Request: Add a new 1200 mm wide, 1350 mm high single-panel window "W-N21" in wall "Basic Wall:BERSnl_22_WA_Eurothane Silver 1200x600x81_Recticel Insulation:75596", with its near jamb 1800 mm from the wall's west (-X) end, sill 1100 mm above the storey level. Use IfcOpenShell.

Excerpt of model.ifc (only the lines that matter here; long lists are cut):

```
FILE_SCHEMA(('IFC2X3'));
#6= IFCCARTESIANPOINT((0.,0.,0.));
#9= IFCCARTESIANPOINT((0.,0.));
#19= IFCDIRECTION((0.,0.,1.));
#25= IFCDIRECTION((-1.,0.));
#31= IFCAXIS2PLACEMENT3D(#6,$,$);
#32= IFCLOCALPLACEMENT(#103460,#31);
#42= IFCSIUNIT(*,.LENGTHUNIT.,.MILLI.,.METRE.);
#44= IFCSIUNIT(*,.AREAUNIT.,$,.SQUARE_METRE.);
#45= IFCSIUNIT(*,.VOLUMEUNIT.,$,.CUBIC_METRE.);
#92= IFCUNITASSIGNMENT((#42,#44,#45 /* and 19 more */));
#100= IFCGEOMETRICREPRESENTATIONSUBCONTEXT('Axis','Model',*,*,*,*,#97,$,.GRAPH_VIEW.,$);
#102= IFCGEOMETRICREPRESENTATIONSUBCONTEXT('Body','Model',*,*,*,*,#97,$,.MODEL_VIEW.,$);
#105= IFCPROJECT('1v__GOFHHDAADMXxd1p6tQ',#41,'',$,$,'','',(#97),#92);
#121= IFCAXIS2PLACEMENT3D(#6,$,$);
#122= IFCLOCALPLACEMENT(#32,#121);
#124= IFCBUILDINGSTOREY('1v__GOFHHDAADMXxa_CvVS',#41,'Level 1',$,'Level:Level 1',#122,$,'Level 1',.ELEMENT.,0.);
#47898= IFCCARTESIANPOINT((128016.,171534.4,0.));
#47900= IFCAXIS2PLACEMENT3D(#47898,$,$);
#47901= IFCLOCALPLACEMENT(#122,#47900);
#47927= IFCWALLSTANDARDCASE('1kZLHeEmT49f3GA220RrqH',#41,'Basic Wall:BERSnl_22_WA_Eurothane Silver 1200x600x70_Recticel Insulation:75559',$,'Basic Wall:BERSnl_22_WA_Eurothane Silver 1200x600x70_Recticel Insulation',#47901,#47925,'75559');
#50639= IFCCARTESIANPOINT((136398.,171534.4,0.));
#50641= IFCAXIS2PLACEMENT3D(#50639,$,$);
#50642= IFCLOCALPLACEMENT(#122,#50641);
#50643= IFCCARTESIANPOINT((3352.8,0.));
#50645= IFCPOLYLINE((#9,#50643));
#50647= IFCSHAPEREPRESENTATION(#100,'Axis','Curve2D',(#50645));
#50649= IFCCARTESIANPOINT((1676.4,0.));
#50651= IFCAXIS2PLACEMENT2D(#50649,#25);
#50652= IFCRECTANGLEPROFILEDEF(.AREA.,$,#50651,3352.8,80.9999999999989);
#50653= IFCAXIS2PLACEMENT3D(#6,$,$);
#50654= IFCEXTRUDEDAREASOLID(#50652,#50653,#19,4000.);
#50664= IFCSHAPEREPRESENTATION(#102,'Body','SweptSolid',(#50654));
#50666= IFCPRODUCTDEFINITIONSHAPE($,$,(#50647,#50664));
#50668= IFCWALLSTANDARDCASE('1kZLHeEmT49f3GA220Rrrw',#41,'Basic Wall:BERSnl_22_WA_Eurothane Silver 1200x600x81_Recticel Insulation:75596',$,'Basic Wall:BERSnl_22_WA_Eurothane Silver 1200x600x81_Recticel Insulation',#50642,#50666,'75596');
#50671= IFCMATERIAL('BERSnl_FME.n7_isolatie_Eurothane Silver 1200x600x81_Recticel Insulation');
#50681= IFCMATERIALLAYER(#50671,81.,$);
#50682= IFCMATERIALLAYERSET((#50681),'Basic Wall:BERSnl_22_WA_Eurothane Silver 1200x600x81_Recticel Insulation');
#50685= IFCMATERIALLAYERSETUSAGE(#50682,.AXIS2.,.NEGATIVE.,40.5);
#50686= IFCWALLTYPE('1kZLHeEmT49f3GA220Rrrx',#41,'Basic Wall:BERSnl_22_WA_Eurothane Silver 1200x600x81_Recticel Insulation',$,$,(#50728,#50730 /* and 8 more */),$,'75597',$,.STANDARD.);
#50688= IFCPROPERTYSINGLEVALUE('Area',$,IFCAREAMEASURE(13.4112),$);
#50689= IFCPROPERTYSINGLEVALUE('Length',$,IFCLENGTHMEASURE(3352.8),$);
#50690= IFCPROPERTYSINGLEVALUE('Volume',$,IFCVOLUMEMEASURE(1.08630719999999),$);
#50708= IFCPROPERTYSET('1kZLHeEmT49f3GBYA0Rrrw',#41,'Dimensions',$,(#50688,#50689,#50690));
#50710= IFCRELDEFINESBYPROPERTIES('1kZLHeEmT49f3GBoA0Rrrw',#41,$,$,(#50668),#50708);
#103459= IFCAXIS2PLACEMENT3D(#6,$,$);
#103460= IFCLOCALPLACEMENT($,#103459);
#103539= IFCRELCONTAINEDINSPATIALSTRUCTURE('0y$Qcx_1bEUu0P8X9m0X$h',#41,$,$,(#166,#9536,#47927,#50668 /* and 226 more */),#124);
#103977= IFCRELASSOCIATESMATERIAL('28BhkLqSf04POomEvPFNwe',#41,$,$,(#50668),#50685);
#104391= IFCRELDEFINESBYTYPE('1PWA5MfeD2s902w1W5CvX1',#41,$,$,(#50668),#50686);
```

```python
import numpy as np
import ifcopenshell
import ifcopenshell.api.feature
import ifcopenshell.api.geometry
import ifcopenshell.api.pset
import ifcopenshell.api.root
import ifcopenshell.api.spatial
import ifcopenshell.api.type
import ifcopenshell.geom
import ifcopenshell.util.element
import ifcopenshell.util.placement
import ifcopenshell.util.representation
import ifcopenshell.util.shape
import ifcopenshell.util.unit

model = ifcopenshell.open("model.ifc")
unit_scale = ifcopenshell.util.unit.calculate_unit_scale(model)
area_scale = ifcopenshell.util.unit.calculate_unit_scale(model, "AREAUNIT")
volume_scale = ifcopenshell.util.unit.calculate_unit_scale(model, "VOLUMEUNIT")
settings = ifcopenshell.geom.settings()


def volume(element):
    """Net volume in cubic metres, openings subtracted."""
    shape = ifcopenshell.geom.create_shape(settings, element)
    return ifcopenshell.util.shape.get_volume(shape.geometry)


wall = model.by_guid("1kZLHeEmT49f3GA220Rrrw")
storey = ifcopenshell.util.element.get_container(wall, ifc_class="IfcBuildingStorey")
context = ifcopenshell.util.representation.get_context(model, "Model", "Body", "MODEL_VIEW")
before = volume(wall)

width, height, from_end, sill = 1.2, 1.35, 1.8, 1.1  # metres

# The wall runs along its own X axis, and the end named is its -X end.
wall_shape = ifcopenshell.geom.create_shape(settings, wall)
x, y, z = ifcopenshell.util.shape.get_vertices(wall_shape.geometry).T
start = x.min() + from_end
face, thickness = float(y.min()), float(y.max() - y.min())
wall_matrix = ifcopenshell.util.placement.get_local_placement(wall.ObjectPlacement)
level = ifcopenshell.util.placement.get_local_placement(storey.ObjectPlacement)[2, 3]


def in_wall(x, y):
    """Placement at x, y metres in the wall's axes, at sill height."""
    matrix = wall_matrix.copy()
    matrix[:, 3] = wall_matrix @ np.array([x / unit_scale, y / unit_scale, 0.0, 1.0])
    matrix[2, 3] = level + sill / unit_scale
    return matrix


# Opening: a box that overshoots both wall faces by 50 mm.
opening = ifcopenshell.api.root.create_entity(model, ifc_class="IfcOpeningElement")
box = ifcopenshell.api.geometry.add_wall_representation(
    model, context=context, length=width, height=height, thickness=thickness + 0.1
)
ifcopenshell.api.geometry.assign_representation(model, product=opening, representation=box)
ifcopenshell.api.geometry.edit_object_placement(model, product=opening, matrix=in_wall(start, face - 0.05), is_si=False)
ifcopenshell.api.feature.add_feature(model, feature=opening, element=wall)

window = ifcopenshell.api.root.create_entity(model, ifc_class="IfcWindow", name="W-N21")
window.OverallWidth, window.OverallHeight = width / unit_scale, height / unit_scale
body = ifcopenshell.api.geometry.add_window_representation(
    model,
    context=context,
    overall_width=window.OverallWidth,
    overall_height=window.OverallHeight,
    partition_type="SINGLE_PANEL",
)
ifcopenshell.api.geometry.assign_representation(model, product=window, representation=body)
ifcopenshell.api.spatial.assign_container(model, products=[window], relating_structure=storey)
fills = ifcopenshell.api.feature.add_filling(model, opening=opening, element=window)
fills.OwnerHistory = window.OwnerHistory  # required in IFC2X3

# IFC2X3 keeps the operation on the window style.
style = ifcopenshell.api.root.create_entity(model, ifc_class="IfcWindowStyle", name="W-N21")
style.OperationType, style.ConstructionType = "SINGLE_PANEL", "NOTDEFINED"
style.ParameterTakesPrecedence = style.Sizeable = False
ifcopenshell.api.type.assign_type(model, related_objects=[window], relating_type=style)

# Centre the window in the wall's thickness.
ifcopenshell.api.geometry.edit_object_placement(model, product=window, matrix=in_wall(start, face), is_si=False)
window_shape = ifcopenshell.geom.create_shape(settings, window)
depth = ifcopenshell.util.shape.get_vertices(window_shape.geometry)[:, 1]
offset = face + thickness / 2 - (depth.min() + depth.max()) / 2
ifcopenshell.api.geometry.edit_object_placement(model, product=window, matrix=in_wall(start, offset), is_si=False)

after = volume(wall)

# Update the wall's stored quantities.
pset = model.by_id(ifcopenshell.util.element.get_pset(wall, "Dimensions", should_inherit=False)["id"])
ifcopenshell.api.pset.edit_pset(model, pset=pset, properties={
    "Area": model.create_entity("IfcAreaMeasure", after / thickness / area_scale),
    "Volume": model.create_entity("IfcVolumeMeasure", after / volume_scale),
})

print(f"wall volume {before:.3f} -> {after:.3f} m3")

model.write("model_edited.ifc")
```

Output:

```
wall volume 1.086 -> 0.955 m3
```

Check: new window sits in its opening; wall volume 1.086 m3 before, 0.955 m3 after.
